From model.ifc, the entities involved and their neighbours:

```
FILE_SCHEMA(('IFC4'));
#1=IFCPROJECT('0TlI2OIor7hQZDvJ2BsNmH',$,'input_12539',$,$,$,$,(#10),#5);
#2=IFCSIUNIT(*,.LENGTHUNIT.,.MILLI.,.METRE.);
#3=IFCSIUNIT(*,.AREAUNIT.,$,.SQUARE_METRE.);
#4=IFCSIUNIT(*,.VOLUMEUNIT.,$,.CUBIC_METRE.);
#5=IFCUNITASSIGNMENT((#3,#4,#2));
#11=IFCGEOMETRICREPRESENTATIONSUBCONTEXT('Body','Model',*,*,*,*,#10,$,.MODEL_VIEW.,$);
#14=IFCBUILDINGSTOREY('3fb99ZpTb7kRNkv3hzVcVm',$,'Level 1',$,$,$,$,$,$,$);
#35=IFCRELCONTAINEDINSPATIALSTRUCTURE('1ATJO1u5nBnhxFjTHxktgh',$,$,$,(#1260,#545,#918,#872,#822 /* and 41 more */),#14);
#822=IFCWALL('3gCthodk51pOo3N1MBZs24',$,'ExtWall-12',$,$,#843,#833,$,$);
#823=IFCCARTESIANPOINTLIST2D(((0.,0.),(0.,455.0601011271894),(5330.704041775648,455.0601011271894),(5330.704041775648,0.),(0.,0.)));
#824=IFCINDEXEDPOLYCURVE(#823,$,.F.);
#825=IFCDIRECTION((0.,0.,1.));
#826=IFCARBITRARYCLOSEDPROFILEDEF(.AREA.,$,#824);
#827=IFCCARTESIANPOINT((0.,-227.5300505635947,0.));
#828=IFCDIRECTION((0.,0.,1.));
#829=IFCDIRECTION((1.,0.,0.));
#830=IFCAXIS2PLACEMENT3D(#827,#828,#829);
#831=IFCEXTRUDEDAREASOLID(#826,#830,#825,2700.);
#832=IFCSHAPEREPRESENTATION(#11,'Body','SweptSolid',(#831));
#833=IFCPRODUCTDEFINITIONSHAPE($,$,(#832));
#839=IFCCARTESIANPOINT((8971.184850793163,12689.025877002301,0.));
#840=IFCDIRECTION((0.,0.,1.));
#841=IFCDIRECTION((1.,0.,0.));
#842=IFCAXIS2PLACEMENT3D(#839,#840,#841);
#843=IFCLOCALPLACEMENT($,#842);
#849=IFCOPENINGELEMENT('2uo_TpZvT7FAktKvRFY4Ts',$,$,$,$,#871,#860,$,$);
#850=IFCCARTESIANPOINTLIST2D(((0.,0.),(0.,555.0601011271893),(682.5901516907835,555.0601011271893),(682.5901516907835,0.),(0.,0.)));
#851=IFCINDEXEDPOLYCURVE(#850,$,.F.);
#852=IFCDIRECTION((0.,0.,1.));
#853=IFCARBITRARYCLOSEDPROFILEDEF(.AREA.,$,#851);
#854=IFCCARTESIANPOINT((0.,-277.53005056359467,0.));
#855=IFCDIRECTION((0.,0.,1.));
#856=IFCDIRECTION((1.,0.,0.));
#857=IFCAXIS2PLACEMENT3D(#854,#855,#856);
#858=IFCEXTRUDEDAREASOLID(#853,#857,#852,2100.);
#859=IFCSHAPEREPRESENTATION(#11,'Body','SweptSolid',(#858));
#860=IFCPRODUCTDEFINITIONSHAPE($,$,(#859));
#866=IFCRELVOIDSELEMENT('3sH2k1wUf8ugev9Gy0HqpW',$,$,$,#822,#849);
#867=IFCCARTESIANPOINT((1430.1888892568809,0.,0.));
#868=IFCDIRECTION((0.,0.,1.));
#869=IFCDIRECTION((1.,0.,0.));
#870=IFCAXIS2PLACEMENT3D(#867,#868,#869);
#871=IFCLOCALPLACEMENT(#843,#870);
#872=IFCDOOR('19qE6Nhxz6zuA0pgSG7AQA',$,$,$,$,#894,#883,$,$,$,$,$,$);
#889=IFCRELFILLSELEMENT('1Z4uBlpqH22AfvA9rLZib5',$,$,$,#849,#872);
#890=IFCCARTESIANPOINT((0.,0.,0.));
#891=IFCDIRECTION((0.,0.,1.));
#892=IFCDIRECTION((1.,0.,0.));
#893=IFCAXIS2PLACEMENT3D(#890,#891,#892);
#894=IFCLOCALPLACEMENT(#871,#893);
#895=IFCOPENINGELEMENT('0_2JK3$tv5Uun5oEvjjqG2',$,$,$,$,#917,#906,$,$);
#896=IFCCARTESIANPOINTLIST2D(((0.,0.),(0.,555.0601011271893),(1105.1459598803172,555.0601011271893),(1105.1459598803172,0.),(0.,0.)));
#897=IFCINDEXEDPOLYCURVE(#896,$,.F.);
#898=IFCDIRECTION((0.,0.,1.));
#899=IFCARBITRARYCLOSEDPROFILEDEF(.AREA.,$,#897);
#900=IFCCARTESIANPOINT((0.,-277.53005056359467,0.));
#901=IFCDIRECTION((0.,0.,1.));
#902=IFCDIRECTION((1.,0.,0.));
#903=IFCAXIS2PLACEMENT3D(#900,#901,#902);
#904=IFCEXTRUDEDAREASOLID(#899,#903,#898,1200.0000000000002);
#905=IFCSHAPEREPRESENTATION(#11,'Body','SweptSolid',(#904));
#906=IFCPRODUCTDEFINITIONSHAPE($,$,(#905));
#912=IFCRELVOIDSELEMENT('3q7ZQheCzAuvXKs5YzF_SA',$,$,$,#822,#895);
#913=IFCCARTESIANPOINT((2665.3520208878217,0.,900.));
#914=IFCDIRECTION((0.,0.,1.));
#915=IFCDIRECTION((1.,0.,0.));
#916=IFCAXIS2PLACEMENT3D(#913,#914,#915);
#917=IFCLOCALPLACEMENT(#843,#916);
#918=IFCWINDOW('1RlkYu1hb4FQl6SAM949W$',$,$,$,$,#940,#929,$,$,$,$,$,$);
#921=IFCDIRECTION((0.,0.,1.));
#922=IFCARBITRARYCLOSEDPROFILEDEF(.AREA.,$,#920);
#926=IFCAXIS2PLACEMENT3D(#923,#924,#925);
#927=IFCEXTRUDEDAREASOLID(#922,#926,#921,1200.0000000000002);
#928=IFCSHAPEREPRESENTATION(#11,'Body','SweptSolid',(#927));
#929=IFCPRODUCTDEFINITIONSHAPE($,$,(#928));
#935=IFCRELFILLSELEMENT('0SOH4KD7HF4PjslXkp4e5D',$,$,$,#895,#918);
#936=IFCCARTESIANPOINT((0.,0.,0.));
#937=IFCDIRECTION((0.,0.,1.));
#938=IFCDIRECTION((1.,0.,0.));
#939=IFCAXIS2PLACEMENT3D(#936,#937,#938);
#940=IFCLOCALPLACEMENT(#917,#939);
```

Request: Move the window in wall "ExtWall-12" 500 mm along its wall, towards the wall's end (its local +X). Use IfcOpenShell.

```python
import ifcopenshell
import ifcopenshell.api.geometry
import ifcopenshell.util.placement

model = ifcopenshell.open("model.ifc")

window = model.by_guid("1RlkYu1hb4FQl6SAM949W$")
opening = window.FillsVoids[0].RelatingOpeningElement
wall = opening.VoidsElements[0].RelatingBuildingElement

wall_matrix = ifcopenshell.util.placement.get_local_placement(wall.ObjectPlacement)
shift = wall_matrix[:3, 0] * 500.0
before = ifcopenshell.util.placement.get_local_placement(window.ObjectPlacement)[:3, 3].copy()

# The window is placed relative to its opening, so it follows when the opening moves.
matrix = ifcopenshell.util.placement.get_local_placement(opening.ObjectPlacement)
matrix[:3, 3] += shift
ifcopenshell.api.geometry.edit_object_placement(
    model, product=opening, matrix=matrix, is_si=False, should_transform_children=True
)

after = ifcopenshell.util.placement.get_local_placement(window.ObjectPlacement)[:3, 3]
print("window moved by", (after - before).round(3) + 0.0)

model.write("model_edited.ifc")
```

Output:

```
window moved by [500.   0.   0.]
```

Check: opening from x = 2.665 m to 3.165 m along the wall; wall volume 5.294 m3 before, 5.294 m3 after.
